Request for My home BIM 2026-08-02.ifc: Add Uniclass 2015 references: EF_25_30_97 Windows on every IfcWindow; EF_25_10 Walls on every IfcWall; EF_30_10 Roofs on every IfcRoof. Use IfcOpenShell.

First a look at what the model holds.

```python
import ifcopenshell

model = ifcopenshell.open("My home BIM 2026-08-02.ifc")
print(model.schema)
print("classifications:", [c.Name for c in model.by_type("IfcClassification")])
for ifc_class in ("IfcDoor", "IfcRoof", "IfcStair", "IfcWall", "IfcWindow"):
    print(ifc_class, len(model.by_type(ifc_class)))
```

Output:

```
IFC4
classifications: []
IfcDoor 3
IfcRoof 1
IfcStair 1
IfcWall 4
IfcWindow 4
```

```python
import ifcopenshell
import ifcopenshell.api.classification

model = ifcopenshell.open("My home BIM 2026-08-02.ifc")

system = ifcopenshell.api.classification.add_classification(model, classification="Uniclass 2015")

codes = {
    "IfcWindow": ("EF_25_30_97", "Windows"),
    "IfcWall": ("EF_25_10", "Walls"),
    "IfcRoof": ("EF_30_10", "Roofs"),
}
for ifc_class, (code, name) in codes.items():
    products = model.by_type(ifc_class)
    ifcopenshell.api.classification.add_reference(
        model, products=products, classification=system, identification=code, name=name
    )
    print(code, len(products))

model.write("My home BIM 2026-08-02_edited.ifc")
```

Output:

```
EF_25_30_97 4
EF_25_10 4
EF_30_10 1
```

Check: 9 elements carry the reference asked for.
